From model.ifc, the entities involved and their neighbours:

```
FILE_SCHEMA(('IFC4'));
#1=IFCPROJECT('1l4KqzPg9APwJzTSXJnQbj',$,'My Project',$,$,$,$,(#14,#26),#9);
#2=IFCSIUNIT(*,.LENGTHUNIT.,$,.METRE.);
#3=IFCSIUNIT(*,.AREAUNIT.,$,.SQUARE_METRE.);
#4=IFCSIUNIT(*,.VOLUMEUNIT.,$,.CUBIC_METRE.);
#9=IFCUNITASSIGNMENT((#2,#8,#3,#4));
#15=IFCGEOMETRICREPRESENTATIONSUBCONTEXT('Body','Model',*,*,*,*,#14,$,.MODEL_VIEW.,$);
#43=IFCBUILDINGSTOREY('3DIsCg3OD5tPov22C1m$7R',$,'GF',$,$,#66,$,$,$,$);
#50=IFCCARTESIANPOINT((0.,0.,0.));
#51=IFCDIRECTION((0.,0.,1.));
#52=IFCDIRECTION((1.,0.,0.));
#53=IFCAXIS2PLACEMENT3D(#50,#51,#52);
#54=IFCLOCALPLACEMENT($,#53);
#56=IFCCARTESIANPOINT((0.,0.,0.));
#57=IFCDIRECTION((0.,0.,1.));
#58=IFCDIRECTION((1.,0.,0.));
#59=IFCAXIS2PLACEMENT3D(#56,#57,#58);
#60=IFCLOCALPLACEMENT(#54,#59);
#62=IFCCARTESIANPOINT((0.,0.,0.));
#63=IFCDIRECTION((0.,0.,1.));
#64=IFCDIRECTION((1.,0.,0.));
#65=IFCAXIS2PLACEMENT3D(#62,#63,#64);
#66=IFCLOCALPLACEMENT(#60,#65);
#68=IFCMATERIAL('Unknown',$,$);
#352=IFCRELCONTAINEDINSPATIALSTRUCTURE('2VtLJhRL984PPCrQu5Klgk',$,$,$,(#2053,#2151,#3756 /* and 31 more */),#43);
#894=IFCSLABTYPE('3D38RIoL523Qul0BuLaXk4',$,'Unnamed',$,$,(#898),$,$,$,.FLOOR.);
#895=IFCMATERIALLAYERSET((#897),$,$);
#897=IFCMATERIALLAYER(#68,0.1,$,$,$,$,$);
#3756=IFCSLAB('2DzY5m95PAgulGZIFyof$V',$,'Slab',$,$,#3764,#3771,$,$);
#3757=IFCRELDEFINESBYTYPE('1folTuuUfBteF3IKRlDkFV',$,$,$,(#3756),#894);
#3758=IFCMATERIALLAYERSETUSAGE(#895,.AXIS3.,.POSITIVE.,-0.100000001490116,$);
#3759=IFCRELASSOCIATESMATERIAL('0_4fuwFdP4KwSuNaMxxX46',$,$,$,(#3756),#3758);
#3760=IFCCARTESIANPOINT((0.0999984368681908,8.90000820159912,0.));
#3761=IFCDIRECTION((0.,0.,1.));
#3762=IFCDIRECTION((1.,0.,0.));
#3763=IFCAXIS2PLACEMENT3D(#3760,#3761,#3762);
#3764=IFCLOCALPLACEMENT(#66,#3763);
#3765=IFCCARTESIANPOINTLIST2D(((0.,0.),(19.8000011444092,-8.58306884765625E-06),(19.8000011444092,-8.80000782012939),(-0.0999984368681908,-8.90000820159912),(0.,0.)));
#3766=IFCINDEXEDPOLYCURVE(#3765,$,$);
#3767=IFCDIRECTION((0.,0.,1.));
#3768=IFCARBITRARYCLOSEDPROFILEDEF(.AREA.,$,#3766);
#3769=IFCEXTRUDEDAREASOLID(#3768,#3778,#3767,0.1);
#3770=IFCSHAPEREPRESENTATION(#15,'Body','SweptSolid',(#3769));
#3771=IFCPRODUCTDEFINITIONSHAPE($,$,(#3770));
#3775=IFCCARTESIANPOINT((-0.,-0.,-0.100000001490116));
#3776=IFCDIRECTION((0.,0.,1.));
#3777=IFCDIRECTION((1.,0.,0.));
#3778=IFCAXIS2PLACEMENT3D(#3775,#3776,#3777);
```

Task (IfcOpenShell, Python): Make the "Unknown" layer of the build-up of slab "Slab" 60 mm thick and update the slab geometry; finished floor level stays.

```python
import ifcopenshell
import ifcopenshell.util.element
import ifcopenshell.util.representation
import ifcopenshell.util.unit

model = ifcopenshell.open("model.ifc")
unit_scale = ifcopenshell.util.unit.calculate_unit_scale(model)

layer_set = model.by_id(895)
layer = next(l for l in layer_set.MaterialLayers if l.Material and l.Material.Name == "Unknown")
change = 0.06 / unit_scale - layer.LayerThickness
layer.LayerThickness += change

# Geometry does not follow the layer set by itself.
slabs = [e for e in ifcopenshell.util.element.get_elements_by_material(model, layer_set) if e.is_a("IfcSlab")]
for slab in sorted(slabs, key=lambda e: e.id()):
    body = ifcopenshell.util.representation.get_representation(slab, "Model", "Body")
    solid = body.Items[0]
    old_depth = solid.Depth
    solid.Depth += change
    # Extruded upwards: lower the start of the extrusion so the top stays.
    x, y, z = solid.Position.Location.Coordinates
    solid.Position.Location = model.createIfcCartesianPoint((x, y, z - change))
    print(slab.id(), f"{old_depth:g} -> {solid.Depth:g}")

# The layers are counted up from the underside, which has moved.
for usage in {ifcopenshell.util.element.get_material(slab) for slab in slabs}:
    usage.OffsetFromReferenceLine -= change

model.write("model-out.ifc")
```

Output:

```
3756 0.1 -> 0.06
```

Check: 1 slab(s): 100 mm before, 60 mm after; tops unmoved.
